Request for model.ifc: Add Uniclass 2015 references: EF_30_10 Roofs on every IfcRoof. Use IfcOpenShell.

First a look at what the model holds.

```python
import ifcopenshell

model = ifcopenshell.open("model.ifc")
print(model.schema)
print("classifications:", [c.Name for c in model.by_type("IfcClassification")])
for ifc_class in ("IfcDoor", "IfcRoof", "IfcStair", "IfcWall", "IfcWindow"):
    print(ifc_class, len(model.by_type(ifc_class)))
```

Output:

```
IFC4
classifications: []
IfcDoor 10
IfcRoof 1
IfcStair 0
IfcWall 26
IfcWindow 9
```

```python
import ifcopenshell
import ifcopenshell.api.classification

model = ifcopenshell.open("model.ifc")

system = ifcopenshell.api.classification.add_classification(model, classification="Uniclass 2015")

codes = {
    "IfcRoof": ("EF_30_10", "Roofs"),
}
for ifc_class, (code, name) in codes.items():
    products = model.by_type(ifc_class)
    ifcopenshell.api.classification.add_reference(
        model, products=products, classification=system, identification=code, name=name
    )
    print(code, len(products))

model.write("model_updated.ifc")
```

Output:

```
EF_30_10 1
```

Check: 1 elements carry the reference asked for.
